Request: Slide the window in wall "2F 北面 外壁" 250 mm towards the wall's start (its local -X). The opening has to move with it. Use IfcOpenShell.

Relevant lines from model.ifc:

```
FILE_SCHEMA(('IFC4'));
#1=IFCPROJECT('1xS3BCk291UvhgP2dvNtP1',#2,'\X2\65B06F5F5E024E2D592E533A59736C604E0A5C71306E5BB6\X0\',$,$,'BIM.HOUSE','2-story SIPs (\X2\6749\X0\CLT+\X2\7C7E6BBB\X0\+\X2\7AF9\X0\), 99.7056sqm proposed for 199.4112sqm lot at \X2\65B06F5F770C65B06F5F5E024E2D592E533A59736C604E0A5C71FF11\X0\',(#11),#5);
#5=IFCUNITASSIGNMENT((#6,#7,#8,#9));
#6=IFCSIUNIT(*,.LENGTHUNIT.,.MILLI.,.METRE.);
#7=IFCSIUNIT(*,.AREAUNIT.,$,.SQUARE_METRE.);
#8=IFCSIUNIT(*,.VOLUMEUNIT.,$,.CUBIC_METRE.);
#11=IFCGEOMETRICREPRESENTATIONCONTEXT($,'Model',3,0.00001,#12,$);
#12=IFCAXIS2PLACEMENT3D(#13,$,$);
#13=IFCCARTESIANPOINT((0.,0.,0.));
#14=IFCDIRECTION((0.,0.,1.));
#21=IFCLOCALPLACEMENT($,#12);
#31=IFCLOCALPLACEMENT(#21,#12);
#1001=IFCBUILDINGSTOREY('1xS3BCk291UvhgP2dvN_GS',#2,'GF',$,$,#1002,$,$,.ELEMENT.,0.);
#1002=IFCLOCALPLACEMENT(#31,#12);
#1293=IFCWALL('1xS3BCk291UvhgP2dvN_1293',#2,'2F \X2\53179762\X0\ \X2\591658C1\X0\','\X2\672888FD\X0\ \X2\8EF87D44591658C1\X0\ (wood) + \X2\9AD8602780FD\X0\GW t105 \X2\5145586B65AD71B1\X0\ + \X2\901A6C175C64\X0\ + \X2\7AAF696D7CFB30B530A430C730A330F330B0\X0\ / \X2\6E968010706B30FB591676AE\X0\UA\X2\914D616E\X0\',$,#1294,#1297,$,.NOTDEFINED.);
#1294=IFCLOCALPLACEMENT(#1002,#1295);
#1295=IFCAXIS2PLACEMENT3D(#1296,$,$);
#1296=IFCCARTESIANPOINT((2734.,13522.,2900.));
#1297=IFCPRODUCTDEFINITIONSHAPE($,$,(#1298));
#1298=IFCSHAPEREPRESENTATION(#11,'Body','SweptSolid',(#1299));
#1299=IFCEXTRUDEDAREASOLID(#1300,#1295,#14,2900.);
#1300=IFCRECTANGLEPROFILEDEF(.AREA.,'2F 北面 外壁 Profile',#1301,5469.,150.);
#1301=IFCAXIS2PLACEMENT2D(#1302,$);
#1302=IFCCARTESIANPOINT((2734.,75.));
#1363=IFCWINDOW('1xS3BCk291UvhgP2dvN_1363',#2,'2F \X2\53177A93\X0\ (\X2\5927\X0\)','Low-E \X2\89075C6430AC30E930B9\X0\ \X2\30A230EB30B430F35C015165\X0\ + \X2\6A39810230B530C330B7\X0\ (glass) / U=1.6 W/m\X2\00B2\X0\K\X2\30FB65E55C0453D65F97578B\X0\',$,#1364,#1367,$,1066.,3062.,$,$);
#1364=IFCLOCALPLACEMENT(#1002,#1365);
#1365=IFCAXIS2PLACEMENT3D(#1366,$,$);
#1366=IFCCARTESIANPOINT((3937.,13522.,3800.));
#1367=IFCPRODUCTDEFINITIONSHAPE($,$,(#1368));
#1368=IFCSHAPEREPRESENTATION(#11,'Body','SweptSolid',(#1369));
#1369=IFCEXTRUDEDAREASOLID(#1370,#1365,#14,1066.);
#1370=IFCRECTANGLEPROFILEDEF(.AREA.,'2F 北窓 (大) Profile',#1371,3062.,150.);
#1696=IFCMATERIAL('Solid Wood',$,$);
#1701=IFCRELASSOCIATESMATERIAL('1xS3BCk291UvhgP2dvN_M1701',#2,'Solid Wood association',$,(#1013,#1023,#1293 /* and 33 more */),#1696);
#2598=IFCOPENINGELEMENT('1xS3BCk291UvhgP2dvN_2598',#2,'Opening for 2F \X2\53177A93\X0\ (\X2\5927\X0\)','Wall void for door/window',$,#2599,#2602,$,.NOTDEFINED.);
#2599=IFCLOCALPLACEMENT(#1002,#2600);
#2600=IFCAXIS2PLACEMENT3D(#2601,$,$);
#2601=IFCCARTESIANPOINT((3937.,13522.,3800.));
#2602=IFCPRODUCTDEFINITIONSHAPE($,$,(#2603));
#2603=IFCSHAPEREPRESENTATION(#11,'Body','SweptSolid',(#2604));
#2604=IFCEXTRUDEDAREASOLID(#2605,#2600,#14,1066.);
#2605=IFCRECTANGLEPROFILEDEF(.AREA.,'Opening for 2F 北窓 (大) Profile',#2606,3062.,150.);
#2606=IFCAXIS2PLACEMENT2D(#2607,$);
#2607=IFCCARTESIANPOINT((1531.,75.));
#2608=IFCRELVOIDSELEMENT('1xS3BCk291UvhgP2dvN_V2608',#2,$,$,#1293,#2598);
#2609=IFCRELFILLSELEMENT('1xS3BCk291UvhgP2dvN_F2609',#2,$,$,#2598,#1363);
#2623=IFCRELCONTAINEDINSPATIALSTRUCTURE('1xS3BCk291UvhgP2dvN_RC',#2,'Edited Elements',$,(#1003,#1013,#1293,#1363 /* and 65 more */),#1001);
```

```python
import ifcopenshell
import ifcopenshell.api.geometry
import ifcopenshell.util.placement
import ifcopenshell.util.unit

model = ifcopenshell.open("model.ifc")
unit_scale = ifcopenshell.util.unit.calculate_unit_scale(model)

window = model.by_guid("1xS3BCk291UvhgP2dvN_1363")
opening = window.FillsVoids[0].RelatingOpeningElement
wall = opening.VoidsElements[0].RelatingBuildingElement

wall_matrix = ifcopenshell.util.placement.get_local_placement(wall.ObjectPlacement)
shift = wall_matrix[:3, 0] * -0.25 / unit_scale
before = ifcopenshell.util.placement.get_local_placement(window.ObjectPlacement)[:3, 3].copy()

# The window is not placed relative to its opening, so move both.
for product in (opening, window):
    matrix = ifcopenshell.util.placement.get_local_placement(product.ObjectPlacement)
    matrix[:3, 3] += shift
    ifcopenshell.api.geometry.edit_object_placement(model, product=product, matrix=matrix, is_si=False)

after = ifcopenshell.util.placement.get_local_placement(window.ObjectPlacement)[:3, 3]
print("window moved by", (after - before).round(3) + 0.0)

model.write("model_rev.ifc")
```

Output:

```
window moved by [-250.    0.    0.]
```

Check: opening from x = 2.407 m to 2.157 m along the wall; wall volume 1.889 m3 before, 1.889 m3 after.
